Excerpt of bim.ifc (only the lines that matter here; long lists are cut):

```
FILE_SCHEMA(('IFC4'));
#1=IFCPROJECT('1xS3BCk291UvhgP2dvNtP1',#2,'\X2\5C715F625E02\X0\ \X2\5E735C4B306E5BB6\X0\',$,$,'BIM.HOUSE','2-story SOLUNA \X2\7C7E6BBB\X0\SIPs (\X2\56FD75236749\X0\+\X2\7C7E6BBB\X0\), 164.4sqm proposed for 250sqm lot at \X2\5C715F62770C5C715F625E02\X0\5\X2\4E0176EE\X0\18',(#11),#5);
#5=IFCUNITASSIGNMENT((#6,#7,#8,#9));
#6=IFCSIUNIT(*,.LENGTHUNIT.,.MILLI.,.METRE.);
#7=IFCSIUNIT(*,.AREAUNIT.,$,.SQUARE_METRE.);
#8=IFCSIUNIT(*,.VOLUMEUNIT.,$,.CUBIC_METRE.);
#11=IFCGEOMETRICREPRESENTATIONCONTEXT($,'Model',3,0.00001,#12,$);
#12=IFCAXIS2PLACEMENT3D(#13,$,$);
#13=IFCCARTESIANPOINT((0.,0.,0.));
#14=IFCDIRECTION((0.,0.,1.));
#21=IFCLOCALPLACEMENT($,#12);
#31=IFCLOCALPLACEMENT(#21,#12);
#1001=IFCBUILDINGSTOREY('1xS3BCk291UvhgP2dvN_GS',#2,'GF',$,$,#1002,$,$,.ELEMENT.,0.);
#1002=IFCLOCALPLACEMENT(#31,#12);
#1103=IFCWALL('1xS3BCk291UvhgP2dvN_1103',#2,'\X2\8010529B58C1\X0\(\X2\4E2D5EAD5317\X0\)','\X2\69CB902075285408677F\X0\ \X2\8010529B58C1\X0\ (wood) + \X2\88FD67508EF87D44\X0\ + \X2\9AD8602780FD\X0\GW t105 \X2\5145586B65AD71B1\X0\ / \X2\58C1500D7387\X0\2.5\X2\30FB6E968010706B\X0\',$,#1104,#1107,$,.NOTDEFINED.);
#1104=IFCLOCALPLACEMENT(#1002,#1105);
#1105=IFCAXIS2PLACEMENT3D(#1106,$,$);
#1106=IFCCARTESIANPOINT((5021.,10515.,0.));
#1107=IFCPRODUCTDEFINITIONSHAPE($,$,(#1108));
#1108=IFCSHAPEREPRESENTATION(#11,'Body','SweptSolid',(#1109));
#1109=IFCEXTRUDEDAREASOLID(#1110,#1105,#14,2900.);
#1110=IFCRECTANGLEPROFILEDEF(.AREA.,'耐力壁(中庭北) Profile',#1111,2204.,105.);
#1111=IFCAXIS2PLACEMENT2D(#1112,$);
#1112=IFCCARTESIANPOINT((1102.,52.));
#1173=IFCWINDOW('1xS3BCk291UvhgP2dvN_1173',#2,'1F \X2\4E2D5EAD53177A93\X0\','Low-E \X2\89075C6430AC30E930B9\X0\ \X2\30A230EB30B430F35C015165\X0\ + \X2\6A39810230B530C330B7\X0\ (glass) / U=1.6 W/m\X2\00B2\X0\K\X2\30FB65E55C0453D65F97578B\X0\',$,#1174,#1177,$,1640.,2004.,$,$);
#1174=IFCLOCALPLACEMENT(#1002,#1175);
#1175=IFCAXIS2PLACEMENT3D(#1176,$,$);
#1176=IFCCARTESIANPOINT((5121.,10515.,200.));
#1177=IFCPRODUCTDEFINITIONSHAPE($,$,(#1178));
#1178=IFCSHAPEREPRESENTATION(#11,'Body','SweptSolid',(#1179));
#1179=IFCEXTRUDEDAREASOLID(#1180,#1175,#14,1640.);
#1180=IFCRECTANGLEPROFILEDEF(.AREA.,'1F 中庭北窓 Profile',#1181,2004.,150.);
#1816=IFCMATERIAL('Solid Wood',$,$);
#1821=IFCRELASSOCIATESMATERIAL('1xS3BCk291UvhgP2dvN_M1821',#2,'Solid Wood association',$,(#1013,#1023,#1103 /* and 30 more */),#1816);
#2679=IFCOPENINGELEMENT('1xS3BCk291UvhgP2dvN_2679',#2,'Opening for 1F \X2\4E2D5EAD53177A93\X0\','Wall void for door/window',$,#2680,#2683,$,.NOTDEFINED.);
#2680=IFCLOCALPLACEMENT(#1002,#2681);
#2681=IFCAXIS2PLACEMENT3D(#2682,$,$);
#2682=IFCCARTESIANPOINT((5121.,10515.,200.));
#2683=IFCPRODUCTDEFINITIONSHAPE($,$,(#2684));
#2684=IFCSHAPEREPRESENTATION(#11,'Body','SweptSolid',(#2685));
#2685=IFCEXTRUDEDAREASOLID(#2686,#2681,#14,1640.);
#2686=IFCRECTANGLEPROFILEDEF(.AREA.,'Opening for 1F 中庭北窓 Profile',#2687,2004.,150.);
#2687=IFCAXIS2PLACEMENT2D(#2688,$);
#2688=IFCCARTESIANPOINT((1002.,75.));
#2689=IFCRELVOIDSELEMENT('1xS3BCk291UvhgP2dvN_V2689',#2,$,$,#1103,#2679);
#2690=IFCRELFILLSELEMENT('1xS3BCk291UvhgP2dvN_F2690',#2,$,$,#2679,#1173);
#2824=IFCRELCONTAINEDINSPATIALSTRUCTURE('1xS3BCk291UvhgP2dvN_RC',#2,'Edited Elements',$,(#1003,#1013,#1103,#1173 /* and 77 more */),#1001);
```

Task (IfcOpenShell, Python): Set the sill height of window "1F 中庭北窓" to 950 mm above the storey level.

```python
import numpy as np
import ifcopenshell
import ifcopenshell.api.geometry
import ifcopenshell.geom
import ifcopenshell.util.element
import ifcopenshell.util.placement
import ifcopenshell.util.shape
import ifcopenshell.util.unit

model = ifcopenshell.open("bim.ifc")
unit_scale = ifcopenshell.util.unit.calculate_unit_scale(model)

window = model.by_guid("1xS3BCk291UvhgP2dvN_1173")
opening = window.FillsVoids[0].RelatingOpeningElement
storey = ifcopenshell.util.element.get_container(window, ifc_class="IfcBuildingStorey")
level = ifcopenshell.util.placement.get_local_placement(storey.ObjectPlacement)[2, 3]

# The opening's origin need not be at the sill, so measure its lowest point.
shape = ifcopenshell.geom.create_shape(ifcopenshell.geom.settings(), opening)
bottom = ifcopenshell.util.shape.get_shape_bottom_elevation(shape, shape.geometry) / unit_scale
dz = level + 0.95 / unit_scale - bottom

shift = np.array([0.0, 0.0, dz])
# The window is not placed relative to its opening, so move both.
for product in (opening, window):
    matrix = ifcopenshell.util.placement.get_local_placement(product.ObjectPlacement)
    matrix[:3, 3] += shift
    ifcopenshell.api.geometry.edit_object_placement(model, product=product, matrix=matrix, is_si=False)

print(f"moved by {dz * unit_scale:+.3f} m")

model.write("bim_updated.ifc")
```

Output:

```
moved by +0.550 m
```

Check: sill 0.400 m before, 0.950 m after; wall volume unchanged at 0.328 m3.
